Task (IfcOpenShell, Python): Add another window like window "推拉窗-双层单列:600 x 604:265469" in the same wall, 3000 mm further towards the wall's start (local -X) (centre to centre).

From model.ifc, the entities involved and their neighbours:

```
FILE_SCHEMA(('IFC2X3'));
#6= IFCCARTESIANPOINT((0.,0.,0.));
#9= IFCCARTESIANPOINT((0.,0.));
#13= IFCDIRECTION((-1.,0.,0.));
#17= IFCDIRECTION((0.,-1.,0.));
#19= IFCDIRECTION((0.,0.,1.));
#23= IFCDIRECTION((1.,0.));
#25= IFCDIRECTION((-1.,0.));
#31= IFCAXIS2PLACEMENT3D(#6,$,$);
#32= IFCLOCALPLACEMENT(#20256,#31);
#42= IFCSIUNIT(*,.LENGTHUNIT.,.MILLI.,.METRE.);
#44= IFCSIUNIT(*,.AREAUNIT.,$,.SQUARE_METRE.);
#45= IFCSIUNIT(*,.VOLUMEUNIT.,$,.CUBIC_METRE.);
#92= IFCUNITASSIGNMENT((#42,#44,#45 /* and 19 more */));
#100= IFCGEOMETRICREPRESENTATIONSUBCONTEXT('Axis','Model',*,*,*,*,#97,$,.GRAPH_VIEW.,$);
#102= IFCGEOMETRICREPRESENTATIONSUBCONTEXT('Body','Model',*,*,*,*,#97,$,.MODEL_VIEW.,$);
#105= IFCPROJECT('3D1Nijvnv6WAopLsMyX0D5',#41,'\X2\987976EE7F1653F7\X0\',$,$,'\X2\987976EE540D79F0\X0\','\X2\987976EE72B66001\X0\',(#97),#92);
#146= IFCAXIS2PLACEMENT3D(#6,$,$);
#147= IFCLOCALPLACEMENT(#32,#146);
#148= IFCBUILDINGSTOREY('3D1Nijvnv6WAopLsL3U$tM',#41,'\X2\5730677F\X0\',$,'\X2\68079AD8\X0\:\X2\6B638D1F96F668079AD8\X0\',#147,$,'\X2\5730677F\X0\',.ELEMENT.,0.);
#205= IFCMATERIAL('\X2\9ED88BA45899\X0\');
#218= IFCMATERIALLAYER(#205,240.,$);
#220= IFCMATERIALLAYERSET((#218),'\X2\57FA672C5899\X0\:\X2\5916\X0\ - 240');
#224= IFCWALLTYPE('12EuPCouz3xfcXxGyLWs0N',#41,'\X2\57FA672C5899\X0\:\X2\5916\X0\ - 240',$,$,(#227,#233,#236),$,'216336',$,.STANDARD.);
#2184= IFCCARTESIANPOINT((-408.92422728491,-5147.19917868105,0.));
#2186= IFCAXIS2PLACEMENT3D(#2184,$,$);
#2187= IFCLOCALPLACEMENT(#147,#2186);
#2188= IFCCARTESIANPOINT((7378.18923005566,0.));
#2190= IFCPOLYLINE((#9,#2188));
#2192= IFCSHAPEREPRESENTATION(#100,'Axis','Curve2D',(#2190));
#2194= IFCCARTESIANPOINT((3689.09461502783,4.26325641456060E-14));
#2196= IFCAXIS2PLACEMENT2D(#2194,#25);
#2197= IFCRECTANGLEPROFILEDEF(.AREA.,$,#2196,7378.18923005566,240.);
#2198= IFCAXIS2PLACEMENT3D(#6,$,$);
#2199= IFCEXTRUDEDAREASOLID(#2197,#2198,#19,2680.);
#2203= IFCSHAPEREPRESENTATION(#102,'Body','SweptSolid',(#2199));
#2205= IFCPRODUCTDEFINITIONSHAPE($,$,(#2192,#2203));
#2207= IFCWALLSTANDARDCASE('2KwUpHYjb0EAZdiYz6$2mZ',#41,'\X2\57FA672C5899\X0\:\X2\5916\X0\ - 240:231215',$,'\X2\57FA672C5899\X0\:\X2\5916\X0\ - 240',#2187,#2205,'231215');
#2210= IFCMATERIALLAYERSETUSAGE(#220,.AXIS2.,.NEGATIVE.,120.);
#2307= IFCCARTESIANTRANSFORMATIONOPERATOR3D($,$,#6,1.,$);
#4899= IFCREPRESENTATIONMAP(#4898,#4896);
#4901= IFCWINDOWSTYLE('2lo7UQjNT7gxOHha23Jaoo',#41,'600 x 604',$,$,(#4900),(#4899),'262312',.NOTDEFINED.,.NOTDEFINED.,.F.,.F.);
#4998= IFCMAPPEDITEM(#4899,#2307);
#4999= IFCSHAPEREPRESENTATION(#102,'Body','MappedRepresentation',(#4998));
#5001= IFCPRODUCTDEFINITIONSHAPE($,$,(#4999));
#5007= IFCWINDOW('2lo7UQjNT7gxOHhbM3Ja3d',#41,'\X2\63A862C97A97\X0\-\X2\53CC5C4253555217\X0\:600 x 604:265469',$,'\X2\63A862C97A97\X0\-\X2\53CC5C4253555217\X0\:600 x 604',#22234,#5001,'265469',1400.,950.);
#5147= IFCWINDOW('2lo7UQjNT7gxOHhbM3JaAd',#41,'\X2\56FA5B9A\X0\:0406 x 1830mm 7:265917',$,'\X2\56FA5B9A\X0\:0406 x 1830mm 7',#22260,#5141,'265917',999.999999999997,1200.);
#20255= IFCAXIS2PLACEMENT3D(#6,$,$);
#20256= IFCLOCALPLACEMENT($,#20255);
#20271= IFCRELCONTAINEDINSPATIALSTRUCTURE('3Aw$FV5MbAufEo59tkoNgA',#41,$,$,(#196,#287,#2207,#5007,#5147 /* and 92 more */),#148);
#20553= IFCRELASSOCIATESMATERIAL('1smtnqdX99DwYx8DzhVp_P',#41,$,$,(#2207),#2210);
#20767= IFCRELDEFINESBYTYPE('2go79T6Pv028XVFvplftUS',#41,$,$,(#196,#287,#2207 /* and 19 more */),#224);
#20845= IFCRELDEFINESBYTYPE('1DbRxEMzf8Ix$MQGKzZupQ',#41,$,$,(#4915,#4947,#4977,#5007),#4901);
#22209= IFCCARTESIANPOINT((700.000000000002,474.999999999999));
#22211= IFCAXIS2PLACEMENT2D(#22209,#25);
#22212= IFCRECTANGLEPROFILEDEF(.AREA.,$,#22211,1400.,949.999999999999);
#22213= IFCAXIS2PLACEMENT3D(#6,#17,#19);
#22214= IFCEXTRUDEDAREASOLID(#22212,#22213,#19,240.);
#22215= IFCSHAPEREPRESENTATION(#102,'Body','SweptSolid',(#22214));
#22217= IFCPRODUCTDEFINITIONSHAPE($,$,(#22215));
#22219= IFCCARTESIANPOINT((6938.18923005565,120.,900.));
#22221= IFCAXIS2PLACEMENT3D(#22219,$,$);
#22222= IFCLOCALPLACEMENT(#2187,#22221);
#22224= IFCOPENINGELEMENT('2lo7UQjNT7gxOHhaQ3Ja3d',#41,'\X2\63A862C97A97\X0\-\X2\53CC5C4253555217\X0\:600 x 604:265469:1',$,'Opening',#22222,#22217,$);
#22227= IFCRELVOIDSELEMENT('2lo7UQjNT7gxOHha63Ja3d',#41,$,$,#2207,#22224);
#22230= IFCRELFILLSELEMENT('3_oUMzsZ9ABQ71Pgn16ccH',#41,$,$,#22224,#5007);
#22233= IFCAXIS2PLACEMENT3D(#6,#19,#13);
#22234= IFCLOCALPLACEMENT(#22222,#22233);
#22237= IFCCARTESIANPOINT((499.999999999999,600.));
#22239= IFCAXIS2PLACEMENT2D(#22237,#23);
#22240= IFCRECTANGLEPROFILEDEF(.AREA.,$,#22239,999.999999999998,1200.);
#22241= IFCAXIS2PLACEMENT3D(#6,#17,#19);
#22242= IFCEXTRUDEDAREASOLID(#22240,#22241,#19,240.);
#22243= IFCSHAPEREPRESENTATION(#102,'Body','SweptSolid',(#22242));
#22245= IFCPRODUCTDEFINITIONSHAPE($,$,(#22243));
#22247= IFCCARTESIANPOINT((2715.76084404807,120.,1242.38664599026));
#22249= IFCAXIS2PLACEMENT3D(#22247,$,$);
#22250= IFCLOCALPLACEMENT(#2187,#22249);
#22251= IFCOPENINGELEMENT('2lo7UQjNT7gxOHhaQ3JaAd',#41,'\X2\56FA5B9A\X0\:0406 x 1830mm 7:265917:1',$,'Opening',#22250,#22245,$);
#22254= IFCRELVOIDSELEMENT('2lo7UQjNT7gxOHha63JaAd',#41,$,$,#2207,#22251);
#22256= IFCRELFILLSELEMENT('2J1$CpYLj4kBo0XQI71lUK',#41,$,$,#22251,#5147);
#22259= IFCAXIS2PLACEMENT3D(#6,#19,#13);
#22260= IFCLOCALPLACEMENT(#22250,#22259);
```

```python
import ifcopenshell
import ifcopenshell.api.feature
import ifcopenshell.api.geometry
import ifcopenshell.api.root
import ifcopenshell.geom
import ifcopenshell.util.element
import ifcopenshell.util.placement
import ifcopenshell.util.shape

model = ifcopenshell.open("model.ifc")
settings = ifcopenshell.geom.settings()


def volume(element):
    """Net volume in cubic metres, openings subtracted."""
    shape = ifcopenshell.geom.create_shape(settings, element)
    return ifcopenshell.util.shape.get_volume(shape.geometry)


def reuse_history(source, copy):
    """copy_class also copies each property set's owner history, people and application; keep the originals."""
    for rel in copy.IsDefinedBy:
        if rel.is_a("IfcRelDefinesByProperties") and (history := rel.RelatingPropertyDefinition.OwnerHistory):
            rel.RelatingPropertyDefinition.OwnerHistory = source.OwnerHistory
            ifcopenshell.util.element.remove_deep2(model, history)


window = model.by_id(5007)
opening = window.FillsVoids[0].RelatingOpeningElement
wall = opening.VoidsElements[0].RelatingBuildingElement
before = volume(wall)
shift = ifcopenshell.util.placement.get_local_placement(wall.ObjectPlacement)[:3, 0] * -3000.0

# copy_class copies the void relationship, type, container and properties, but no geometry.
new_opening = ifcopenshell.api.root.copy_class(model, product=opening)
new_opening.Representation = ifcopenshell.util.element.copy_deep(
    model, opening.Representation, exclude=["IfcGeometricRepresentationContext", "IfcRepresentationMap"]
)
new_opening.Name = "推拉窗-双层单列:600 x 604"
new_window = ifcopenshell.api.root.copy_class(model, product=window)
new_window.Representation = ifcopenshell.util.element.copy_deep(
    model, window.Representation, exclude=["IfcGeometricRepresentationContext", "IfcRepresentationMap"]
)
new_window.Name = "推拉窗-双层单列:600 x 604"
new_window.Tag = None
reuse_history(window, new_window)
fills = ifcopenshell.api.feature.add_filling(model, opening=new_opening, element=new_window)
fills.OwnerHistory = new_window.OwnerHistory  # required in IFC2X3

for old, new in ((opening, new_opening), (window, new_window)):
    matrix = ifcopenshell.util.placement.get_local_placement(old.ObjectPlacement)
    matrix[:3, 3] += shift
    ifcopenshell.api.geometry.edit_object_placement(model, product=new, matrix=matrix, is_si=False)

after = volume(wall)

print(f"wall volume {before:.3f} -> {after:.3f} m3")

model.write("model-out.ifc")
```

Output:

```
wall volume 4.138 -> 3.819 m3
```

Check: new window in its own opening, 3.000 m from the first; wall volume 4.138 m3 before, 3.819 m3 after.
